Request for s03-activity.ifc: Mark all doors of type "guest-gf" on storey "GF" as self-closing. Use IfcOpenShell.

First a look at what the model holds.

```python
import ifcopenshell
import ifcopenshell.util.element

model = ifcopenshell.open("s03-activity.ifc")
print(model.schema)
storey = next(s for s in model.by_type("IfcBuildingStorey") if s.Name == "GF")
doors = [e for e in ifcopenshell.util.element.get_decomposition(storey) if e.is_a("IfcDoor")]
seen = {}
for e in doors:
    element_type = ifcopenshell.util.element.get_type(e)
    key = (element_type.Name if element_type != e and element_type else None, ifcopenshell.util.element.get_pset(e, "Pset_DoorCommon", "SelfClosing"))
    seen[key] = seen.get(key, 0) + 1
for (name, value), count in sorted(seen.items(), key=str):
    print(count, "x", name, "|", value)
```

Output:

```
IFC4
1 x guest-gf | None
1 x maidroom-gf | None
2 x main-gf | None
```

```python
import ifcopenshell
import ifcopenshell.api.pset
import ifcopenshell.util.element

model = ifcopenshell.open("s03-activity.ifc")

storey = next(s for s in model.by_type("IfcBuildingStorey") if s.Name == "GF")
doors = [e for e in ifcopenshell.util.element.get_decomposition(storey) if e.is_a("IfcDoor")]

count = 0
for e in doors:
    element_type = ifcopenshell.util.element.get_type(e)
    if element_type in (None, e) or element_type.Name != "guest-gf":
        continue
    # add_pset returns the element's existing set when there is one.
    pset = ifcopenshell.api.pset.add_pset(model, product=e, name="Pset_DoorCommon")
    ifcopenshell.api.pset.edit_pset(model, pset=pset, properties={"SelfClosing": True})
    count += 1

print(count, "doors updated")

model.write("s03-activity-out.ifc")
```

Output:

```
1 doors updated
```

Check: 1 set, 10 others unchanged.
